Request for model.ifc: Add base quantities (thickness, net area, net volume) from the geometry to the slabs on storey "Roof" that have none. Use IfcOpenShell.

First a look at what the model holds.

```python
import ifcopenshell
import ifcopenshell.util.element
import ifcopenshell.util.unit

model = ifcopenshell.open("model.ifc")
print(model.schema)
for unit_type in ("LENGTHUNIT", "AREAUNIT", "VOLUMEUNIT"):
    print(unit_type, ifcopenshell.util.unit.calculate_unit_scale(model, unit_type))
storey = next(s for s in model.by_type("IfcBuildingStorey") if s.Name == "Roof")
slabs = [e for e in ifcopenshell.util.element.get_decomposition(storey) if e.is_a("IfcSlab")]
for e in sorted(slabs, key=lambda e: e.id()):
    print(e.id(), e.is_a(), e.Name, list(ifcopenshell.util.element.get_psets(e, qtos_only=True)), sep=" | ")
```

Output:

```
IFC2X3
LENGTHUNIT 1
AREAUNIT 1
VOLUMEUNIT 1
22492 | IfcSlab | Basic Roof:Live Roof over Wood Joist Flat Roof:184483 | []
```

```python
import ifcopenshell
import ifcopenshell.api.pset
import ifcopenshell.geom
import ifcopenshell.util.element
import ifcopenshell.util.shape
import ifcopenshell.util.unit

model = ifcopenshell.open("model.ifc")
unit_scale = ifcopenshell.util.unit.calculate_unit_scale(model)
area_scale = ifcopenshell.util.unit.calculate_unit_scale(model, "AREAUNIT")
volume_scale = ifcopenshell.util.unit.calculate_unit_scale(model, "VOLUMEUNIT")
settings = ifcopenshell.geom.settings()

storey = next(s for s in model.by_type("IfcBuildingStorey") if s.Name == "Roof")
slabs = [e for e in ifcopenshell.util.element.get_decomposition(storey) if e.is_a("IfcSlab")]

for e in sorted(slabs, key=lambda e: e.id()):
    if ifcopenshell.util.element.get_psets(e, qtos_only=True, should_inherit=False):
        continue
    # Geometry comes back in metres, in the element's own axes.
    shape = ifcopenshell.geom.create_shape(settings, e)
    values = {
        "Width": ifcopenshell.util.shape.get_z(shape.geometry) / unit_scale,
        "NetArea": ifcopenshell.util.shape.get_footprint_area(shape.geometry) / area_scale,
        "NetVolume": ifcopenshell.util.shape.get_volume(shape.geometry) / volume_scale,
    }
    qto = ifcopenshell.api.pset.add_qto(model, product=e, name="BaseQuantities")
    ifcopenshell.api.pset.edit_qto(model, qto=qto, properties=values)
    print(e.id(), {k: round(v, 3) for k, v in values.items()})

model.write("model-out.ifc")
```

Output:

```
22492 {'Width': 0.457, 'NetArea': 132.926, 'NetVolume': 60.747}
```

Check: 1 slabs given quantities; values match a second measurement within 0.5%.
